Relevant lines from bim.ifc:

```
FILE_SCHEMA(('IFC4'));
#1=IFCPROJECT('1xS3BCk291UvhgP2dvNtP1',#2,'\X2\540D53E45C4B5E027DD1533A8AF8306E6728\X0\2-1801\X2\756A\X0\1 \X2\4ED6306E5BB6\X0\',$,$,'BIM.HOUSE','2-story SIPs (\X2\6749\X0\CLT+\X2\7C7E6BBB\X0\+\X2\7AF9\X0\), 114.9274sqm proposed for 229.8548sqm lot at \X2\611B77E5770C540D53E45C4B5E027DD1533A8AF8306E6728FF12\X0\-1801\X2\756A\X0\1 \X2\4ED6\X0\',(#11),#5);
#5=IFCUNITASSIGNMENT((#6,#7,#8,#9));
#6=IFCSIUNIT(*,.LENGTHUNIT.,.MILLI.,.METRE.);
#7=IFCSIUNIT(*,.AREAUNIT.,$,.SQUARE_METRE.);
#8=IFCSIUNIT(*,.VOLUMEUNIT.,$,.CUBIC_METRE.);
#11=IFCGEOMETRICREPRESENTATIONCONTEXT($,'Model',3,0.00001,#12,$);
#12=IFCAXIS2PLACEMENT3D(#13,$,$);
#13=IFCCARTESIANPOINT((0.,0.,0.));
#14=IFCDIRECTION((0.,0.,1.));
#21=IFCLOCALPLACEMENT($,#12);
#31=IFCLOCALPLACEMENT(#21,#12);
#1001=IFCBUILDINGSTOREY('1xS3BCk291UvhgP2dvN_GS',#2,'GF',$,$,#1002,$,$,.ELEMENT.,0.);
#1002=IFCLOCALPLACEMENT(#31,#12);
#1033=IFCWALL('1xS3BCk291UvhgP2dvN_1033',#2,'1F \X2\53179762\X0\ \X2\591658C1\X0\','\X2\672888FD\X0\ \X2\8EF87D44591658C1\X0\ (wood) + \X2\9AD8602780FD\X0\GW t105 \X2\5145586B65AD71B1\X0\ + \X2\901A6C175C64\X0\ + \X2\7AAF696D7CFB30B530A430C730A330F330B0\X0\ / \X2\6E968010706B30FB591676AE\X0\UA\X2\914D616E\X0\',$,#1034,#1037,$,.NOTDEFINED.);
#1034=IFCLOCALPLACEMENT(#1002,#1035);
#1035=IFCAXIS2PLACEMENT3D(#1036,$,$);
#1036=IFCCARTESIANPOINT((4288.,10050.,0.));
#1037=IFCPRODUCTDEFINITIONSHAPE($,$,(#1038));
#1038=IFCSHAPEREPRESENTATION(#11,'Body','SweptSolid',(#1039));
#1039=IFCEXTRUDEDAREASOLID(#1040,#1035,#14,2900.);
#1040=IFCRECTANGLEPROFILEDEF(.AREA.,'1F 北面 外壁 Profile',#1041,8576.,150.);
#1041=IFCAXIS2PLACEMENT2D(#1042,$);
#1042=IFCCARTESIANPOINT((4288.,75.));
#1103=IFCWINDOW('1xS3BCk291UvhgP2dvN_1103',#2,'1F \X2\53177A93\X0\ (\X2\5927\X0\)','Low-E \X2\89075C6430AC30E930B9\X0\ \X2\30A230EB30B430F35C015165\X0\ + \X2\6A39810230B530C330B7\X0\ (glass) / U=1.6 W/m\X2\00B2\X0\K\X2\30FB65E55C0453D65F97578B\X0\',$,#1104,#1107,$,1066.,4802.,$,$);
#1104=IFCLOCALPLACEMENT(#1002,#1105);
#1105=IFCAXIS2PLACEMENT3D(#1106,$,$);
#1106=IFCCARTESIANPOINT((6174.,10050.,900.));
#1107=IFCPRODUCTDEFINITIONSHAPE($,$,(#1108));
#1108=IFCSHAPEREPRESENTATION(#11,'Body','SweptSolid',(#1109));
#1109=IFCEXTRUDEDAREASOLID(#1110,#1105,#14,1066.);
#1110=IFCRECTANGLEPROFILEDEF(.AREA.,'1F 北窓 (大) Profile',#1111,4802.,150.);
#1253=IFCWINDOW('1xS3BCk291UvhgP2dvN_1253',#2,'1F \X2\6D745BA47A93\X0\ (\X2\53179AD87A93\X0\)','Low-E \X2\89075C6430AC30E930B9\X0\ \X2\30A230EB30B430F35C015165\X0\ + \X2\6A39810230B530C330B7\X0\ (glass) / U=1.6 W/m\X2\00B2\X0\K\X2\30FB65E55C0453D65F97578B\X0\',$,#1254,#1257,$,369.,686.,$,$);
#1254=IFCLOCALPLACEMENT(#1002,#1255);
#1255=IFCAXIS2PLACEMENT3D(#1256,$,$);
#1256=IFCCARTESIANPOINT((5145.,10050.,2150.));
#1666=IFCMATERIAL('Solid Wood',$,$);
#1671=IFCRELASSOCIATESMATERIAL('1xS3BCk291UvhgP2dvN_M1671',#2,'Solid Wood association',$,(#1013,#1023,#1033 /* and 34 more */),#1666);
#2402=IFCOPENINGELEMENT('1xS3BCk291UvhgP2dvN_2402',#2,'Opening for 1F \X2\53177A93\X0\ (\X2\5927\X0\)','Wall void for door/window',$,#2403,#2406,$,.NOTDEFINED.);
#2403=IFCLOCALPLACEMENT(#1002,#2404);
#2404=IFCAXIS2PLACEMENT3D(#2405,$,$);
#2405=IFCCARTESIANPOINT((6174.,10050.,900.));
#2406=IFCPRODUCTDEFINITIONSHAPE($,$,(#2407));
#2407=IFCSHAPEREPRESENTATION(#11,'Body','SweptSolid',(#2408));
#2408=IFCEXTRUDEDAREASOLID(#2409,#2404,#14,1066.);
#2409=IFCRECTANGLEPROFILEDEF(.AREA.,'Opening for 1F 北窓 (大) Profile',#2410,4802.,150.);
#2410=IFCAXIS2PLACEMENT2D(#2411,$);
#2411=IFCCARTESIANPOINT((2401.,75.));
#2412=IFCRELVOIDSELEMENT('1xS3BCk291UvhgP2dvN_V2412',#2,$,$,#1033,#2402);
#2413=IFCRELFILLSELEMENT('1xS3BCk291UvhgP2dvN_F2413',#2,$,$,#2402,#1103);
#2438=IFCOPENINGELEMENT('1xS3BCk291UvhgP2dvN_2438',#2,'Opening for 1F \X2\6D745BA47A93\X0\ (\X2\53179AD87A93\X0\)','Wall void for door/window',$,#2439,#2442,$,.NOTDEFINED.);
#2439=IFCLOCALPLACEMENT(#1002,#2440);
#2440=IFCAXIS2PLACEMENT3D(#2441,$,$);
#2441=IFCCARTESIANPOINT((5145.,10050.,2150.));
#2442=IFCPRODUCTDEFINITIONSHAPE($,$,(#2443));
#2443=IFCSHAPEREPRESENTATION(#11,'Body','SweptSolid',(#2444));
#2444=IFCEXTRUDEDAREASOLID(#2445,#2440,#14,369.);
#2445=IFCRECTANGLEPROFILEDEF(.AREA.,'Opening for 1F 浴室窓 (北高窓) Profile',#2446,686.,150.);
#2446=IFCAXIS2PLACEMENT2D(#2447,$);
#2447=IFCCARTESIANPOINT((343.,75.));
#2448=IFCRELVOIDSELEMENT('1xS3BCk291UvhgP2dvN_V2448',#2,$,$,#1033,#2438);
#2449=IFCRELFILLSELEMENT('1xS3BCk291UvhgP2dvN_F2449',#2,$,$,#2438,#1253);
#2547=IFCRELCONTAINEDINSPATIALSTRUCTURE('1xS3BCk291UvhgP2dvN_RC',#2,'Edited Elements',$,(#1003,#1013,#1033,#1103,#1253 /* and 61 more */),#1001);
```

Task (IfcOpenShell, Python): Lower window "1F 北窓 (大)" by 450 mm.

```python
import numpy as np
import ifcopenshell
import ifcopenshell.api.geometry
import ifcopenshell.util.placement
import ifcopenshell.util.unit

model = ifcopenshell.open("bim.ifc")
unit_scale = ifcopenshell.util.unit.calculate_unit_scale(model)

window = model.by_guid("1xS3BCk291UvhgP2dvN_1103")
opening = window.FillsVoids[0].RelatingOpeningElement
dz = -0.45 / unit_scale

shift = np.array([0.0, 0.0, dz])
# The window is not placed relative to its opening, so move both.
for product in (opening, window):
    matrix = ifcopenshell.util.placement.get_local_placement(product.ObjectPlacement)
    matrix[:3, 3] += shift
    ifcopenshell.api.geometry.edit_object_placement(model, product=product, matrix=matrix, is_si=False)

print(f"moved by {dz * unit_scale:+.3f} m")

model.write("bim_updated.ifc")
```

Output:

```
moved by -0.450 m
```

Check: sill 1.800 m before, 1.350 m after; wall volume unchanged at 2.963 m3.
